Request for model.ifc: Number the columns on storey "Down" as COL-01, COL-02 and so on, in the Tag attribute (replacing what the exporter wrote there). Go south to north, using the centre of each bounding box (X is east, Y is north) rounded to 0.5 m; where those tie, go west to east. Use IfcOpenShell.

First a look at what the model holds.

```python
import ifcopenshell
import ifcopenshell.util.element
import ifcopenshell.util.placement

model = ifcopenshell.open("model.ifc")
print(model.schema)
storey = next(s for s in model.by_type("IfcBuildingStorey") if s.Name == "Down")
columns = [e for e in ifcopenshell.util.element.get_decomposition(storey) if e.is_a("IfcColumn")]
for e in sorted(columns, key=lambda e: e.id()):
    origin = ifcopenshell.util.placement.get_local_placement(e.ObjectPlacement)[:3, 3]
    print(e.id(), e.Tag, e.Name, origin.round(2) + 0.0, sep=" | ")
```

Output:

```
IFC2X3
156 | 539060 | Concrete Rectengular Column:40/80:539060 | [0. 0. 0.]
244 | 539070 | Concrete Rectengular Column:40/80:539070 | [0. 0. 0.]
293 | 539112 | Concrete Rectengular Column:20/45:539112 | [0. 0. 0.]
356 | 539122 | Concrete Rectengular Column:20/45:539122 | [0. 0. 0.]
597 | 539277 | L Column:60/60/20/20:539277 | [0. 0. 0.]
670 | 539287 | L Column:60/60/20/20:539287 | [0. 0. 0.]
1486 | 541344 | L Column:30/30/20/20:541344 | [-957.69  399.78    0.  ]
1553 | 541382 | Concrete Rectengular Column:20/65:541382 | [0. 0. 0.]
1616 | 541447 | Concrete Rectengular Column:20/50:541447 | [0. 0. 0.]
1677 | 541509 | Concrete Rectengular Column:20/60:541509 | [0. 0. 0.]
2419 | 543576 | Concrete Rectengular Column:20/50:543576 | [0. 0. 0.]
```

```python
import ifcopenshell
import ifcopenshell.geom
import ifcopenshell.util.element
import ifcopenshell.util.shape

model = ifcopenshell.open("model.ifc")
settings = ifcopenshell.geom.settings()
settings.set("use-world-coords", True)


def centre(element):
    shape = ifcopenshell.geom.create_shape(settings, element)
    return ifcopenshell.util.shape.get_bbox_centroid(shape.geometry)


storey = next(s for s in model.by_type("IfcBuildingStorey") if s.Name == "Down")
columns = [e for e in ifcopenshell.util.element.get_decomposition(storey) if e.is_a("IfcColumn")]

# Insertion points can sit at a corner or the storey origin, so sort by the geometry (in metres).
centres = {e: centre(e) for e in columns}
columns.sort(key=lambda e: (round(centres[e][1] / 0.5), centres[e][0]))

for i, e in enumerate(columns, start=1):
    number = f"COL-{i:02d}"
    e.Tag = number
    print(e.id(), number)

model.write("model_v2.ifc")
```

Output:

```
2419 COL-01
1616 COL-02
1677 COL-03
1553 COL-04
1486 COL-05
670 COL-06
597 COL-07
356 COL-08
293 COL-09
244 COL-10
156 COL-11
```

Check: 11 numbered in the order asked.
